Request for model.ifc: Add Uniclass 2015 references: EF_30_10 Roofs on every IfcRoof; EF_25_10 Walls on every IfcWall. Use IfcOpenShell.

First a look at what the model holds.

```python
import ifcopenshell

model = ifcopenshell.open("model.ifc")
print(model.schema)
print("classifications:", [c.Name for c in model.by_type("IfcClassification")])
for ifc_class in ("IfcDoor", "IfcRoof", "IfcStair", "IfcWall", "IfcWindow"):
    print(ifc_class, len(model.by_type(ifc_class)))
```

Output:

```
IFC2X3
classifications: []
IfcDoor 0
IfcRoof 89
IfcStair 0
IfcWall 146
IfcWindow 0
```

```python
import ifcopenshell
import ifcopenshell.api.classification

model = ifcopenshell.open("model.ifc")

# IFC2X3 requires Source and Edition and has no link from the project to the system.
system = model.create_entity("IfcClassification", Source="NBS", Edition="2015", Name="Uniclass 2015")

codes = {
    "IfcRoof": ("EF_30_10", "Roofs"),
    "IfcWall": ("EF_25_10", "Walls"),
}
for ifc_class, (code, name) in codes.items():
    products = model.by_type(ifc_class)
    ifcopenshell.api.classification.add_reference(
        model, products=products, classification=system, identification=code, name=name
    )
    print(code, len(products))

model.write("model-out.ifc")
```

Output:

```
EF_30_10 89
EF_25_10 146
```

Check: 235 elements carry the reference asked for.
